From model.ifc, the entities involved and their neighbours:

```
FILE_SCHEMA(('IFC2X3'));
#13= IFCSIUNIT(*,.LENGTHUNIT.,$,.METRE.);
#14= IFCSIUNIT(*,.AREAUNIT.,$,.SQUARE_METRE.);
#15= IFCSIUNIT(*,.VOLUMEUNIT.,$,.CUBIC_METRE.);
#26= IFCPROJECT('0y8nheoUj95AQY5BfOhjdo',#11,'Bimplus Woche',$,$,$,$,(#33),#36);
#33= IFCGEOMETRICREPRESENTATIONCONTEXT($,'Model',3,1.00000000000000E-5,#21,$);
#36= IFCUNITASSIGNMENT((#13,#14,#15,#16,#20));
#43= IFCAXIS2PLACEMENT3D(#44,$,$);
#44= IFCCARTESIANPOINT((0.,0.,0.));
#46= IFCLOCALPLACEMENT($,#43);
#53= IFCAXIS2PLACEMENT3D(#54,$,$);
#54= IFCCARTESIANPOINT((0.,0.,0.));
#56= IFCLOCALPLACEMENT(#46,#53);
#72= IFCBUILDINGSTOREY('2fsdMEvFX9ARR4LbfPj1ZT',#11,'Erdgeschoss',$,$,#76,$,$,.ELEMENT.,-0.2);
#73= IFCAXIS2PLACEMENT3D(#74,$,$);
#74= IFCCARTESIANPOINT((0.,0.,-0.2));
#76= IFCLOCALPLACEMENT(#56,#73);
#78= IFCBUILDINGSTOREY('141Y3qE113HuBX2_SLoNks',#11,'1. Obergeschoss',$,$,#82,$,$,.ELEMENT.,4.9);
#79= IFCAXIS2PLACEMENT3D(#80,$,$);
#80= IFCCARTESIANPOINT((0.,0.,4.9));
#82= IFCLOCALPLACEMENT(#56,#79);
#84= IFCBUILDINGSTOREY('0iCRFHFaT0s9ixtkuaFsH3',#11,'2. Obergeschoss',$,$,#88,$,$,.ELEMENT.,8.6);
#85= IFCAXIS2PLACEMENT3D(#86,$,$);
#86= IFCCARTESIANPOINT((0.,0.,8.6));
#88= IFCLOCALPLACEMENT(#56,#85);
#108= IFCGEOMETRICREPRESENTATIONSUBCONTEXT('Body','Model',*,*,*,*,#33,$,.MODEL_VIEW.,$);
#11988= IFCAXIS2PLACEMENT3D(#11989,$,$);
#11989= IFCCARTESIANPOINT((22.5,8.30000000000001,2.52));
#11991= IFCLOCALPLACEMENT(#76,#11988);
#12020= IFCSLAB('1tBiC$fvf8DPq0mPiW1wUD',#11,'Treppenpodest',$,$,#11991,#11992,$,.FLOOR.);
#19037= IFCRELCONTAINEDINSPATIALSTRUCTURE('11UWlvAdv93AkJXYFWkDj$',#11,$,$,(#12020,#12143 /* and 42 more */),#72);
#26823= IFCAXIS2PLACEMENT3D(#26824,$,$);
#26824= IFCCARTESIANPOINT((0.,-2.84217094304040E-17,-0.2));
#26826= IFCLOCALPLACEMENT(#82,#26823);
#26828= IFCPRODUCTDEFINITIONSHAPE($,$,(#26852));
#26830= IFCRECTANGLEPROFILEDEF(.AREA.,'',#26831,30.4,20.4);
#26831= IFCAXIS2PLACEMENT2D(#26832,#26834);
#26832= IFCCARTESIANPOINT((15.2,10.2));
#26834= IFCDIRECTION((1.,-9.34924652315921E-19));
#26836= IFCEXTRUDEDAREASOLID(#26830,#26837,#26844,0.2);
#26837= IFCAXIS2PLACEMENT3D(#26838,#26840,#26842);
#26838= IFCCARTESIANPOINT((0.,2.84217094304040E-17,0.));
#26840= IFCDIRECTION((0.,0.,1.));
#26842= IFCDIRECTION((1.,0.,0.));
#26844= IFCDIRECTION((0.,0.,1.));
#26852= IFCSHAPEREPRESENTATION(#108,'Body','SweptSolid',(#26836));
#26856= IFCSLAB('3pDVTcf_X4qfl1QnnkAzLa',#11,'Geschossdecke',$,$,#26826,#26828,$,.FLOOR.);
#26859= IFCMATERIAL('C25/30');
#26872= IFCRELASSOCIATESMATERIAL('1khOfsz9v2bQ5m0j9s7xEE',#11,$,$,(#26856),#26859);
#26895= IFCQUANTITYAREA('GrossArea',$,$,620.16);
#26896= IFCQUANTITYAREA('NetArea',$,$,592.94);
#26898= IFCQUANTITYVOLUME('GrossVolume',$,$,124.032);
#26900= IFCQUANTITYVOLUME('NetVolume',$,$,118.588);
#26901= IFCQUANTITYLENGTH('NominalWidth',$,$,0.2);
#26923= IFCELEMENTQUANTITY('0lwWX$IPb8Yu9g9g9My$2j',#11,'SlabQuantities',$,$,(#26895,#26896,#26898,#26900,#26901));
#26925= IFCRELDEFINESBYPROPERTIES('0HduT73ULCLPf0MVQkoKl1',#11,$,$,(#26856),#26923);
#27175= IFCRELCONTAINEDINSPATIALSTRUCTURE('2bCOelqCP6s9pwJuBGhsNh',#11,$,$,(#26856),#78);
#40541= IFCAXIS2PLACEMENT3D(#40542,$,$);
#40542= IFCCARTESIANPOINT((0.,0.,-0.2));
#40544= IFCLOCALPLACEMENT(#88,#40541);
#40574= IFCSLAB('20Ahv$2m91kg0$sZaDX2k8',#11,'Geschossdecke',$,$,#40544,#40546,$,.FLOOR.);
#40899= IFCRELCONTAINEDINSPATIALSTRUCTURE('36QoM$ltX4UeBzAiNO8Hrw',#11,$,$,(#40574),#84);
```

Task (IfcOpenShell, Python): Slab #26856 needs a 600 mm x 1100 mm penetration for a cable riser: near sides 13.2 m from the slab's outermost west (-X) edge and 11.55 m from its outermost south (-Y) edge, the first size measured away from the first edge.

```python
import numpy as np
import ifcopenshell
import ifcopenshell.api.feature
import ifcopenshell.api.geometry
import ifcopenshell.api.pset
import ifcopenshell.api.root
import ifcopenshell.geom
import ifcopenshell.util.element
import ifcopenshell.util.placement
import ifcopenshell.util.representation
import ifcopenshell.util.shape
import ifcopenshell.util.unit

model = ifcopenshell.open("model.ifc")
unit_scale = ifcopenshell.util.unit.calculate_unit_scale(model)
area_scale = ifcopenshell.util.unit.calculate_unit_scale(model, "AREAUNIT")
volume_scale = ifcopenshell.util.unit.calculate_unit_scale(model, "VOLUMEUNIT")
settings = ifcopenshell.geom.settings()


def volume(element):
    """Net volume in cubic metres, openings subtracted."""
    shape = ifcopenshell.geom.create_shape(settings, element)
    return ifcopenshell.util.shape.get_volume(shape.geometry)


slab = model.by_guid("3pDVTcf_X4qfl1QnnkAzLa")
before = volume(slab)

# Extent in the slab's own axes, in metres. The edges named are its -X and -Y sides.
slab_shape = ifcopenshell.geom.create_shape(settings, slab)
vertices = ifcopenshell.util.shape.get_vertices(slab_shape.geometry)
x_min, y_min, bottom = vertices.min(axis=0)
top = vertices[:, 2].max()

opening = ifcopenshell.api.root.create_entity(model, ifc_class="IfcOpeningElement", name="Cable riser opening")
context = ifcopenshell.util.representation.get_context(model, "Model", "Body", "MODEL_VIEW")
width, depth = 0.6, 1.1
outline = [(0.0, 0.0), (width, 0.0), (width, depth), (0.0, depth), (0.0, 0.0)]
# Overshoot both faces by 50 mm so the cut is clean.
shape = ifcopenshell.api.geometry.add_slab_representation(
    model, context=context, depth=top - bottom + 0.1, polyline=outline
)
ifcopenshell.api.geometry.assign_representation(model, product=opening, representation=shape)

matrix = ifcopenshell.util.placement.get_local_placement(slab.ObjectPlacement)
matrix[:, 3] = matrix @ np.append(np.array([x_min + 13.2, y_min + 11.55, bottom - 0.05]) / unit_scale, 1.0)
ifcopenshell.api.geometry.edit_object_placement(model, product=opening, matrix=matrix, is_si=False)
ifcopenshell.api.feature.add_feature(model, feature=opening, element=slab)

after = volume(slab)

# Update the slab's stored quantities.
qto = model.by_id(ifcopenshell.util.element.get_pset(slab, "SlabQuantities", should_inherit=False)["id"])
ifcopenshell.api.pset.edit_qto(model, qto=qto, properties={
    "NetArea": after / (top - bottom) / area_scale,
    "NetVolume": after / volume_scale,
})

print(f"slab volume {before:.3f} -> {after:.3f} m3")

model.write("model_updated.ifc")
```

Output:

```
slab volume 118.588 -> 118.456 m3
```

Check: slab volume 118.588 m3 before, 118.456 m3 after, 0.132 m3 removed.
